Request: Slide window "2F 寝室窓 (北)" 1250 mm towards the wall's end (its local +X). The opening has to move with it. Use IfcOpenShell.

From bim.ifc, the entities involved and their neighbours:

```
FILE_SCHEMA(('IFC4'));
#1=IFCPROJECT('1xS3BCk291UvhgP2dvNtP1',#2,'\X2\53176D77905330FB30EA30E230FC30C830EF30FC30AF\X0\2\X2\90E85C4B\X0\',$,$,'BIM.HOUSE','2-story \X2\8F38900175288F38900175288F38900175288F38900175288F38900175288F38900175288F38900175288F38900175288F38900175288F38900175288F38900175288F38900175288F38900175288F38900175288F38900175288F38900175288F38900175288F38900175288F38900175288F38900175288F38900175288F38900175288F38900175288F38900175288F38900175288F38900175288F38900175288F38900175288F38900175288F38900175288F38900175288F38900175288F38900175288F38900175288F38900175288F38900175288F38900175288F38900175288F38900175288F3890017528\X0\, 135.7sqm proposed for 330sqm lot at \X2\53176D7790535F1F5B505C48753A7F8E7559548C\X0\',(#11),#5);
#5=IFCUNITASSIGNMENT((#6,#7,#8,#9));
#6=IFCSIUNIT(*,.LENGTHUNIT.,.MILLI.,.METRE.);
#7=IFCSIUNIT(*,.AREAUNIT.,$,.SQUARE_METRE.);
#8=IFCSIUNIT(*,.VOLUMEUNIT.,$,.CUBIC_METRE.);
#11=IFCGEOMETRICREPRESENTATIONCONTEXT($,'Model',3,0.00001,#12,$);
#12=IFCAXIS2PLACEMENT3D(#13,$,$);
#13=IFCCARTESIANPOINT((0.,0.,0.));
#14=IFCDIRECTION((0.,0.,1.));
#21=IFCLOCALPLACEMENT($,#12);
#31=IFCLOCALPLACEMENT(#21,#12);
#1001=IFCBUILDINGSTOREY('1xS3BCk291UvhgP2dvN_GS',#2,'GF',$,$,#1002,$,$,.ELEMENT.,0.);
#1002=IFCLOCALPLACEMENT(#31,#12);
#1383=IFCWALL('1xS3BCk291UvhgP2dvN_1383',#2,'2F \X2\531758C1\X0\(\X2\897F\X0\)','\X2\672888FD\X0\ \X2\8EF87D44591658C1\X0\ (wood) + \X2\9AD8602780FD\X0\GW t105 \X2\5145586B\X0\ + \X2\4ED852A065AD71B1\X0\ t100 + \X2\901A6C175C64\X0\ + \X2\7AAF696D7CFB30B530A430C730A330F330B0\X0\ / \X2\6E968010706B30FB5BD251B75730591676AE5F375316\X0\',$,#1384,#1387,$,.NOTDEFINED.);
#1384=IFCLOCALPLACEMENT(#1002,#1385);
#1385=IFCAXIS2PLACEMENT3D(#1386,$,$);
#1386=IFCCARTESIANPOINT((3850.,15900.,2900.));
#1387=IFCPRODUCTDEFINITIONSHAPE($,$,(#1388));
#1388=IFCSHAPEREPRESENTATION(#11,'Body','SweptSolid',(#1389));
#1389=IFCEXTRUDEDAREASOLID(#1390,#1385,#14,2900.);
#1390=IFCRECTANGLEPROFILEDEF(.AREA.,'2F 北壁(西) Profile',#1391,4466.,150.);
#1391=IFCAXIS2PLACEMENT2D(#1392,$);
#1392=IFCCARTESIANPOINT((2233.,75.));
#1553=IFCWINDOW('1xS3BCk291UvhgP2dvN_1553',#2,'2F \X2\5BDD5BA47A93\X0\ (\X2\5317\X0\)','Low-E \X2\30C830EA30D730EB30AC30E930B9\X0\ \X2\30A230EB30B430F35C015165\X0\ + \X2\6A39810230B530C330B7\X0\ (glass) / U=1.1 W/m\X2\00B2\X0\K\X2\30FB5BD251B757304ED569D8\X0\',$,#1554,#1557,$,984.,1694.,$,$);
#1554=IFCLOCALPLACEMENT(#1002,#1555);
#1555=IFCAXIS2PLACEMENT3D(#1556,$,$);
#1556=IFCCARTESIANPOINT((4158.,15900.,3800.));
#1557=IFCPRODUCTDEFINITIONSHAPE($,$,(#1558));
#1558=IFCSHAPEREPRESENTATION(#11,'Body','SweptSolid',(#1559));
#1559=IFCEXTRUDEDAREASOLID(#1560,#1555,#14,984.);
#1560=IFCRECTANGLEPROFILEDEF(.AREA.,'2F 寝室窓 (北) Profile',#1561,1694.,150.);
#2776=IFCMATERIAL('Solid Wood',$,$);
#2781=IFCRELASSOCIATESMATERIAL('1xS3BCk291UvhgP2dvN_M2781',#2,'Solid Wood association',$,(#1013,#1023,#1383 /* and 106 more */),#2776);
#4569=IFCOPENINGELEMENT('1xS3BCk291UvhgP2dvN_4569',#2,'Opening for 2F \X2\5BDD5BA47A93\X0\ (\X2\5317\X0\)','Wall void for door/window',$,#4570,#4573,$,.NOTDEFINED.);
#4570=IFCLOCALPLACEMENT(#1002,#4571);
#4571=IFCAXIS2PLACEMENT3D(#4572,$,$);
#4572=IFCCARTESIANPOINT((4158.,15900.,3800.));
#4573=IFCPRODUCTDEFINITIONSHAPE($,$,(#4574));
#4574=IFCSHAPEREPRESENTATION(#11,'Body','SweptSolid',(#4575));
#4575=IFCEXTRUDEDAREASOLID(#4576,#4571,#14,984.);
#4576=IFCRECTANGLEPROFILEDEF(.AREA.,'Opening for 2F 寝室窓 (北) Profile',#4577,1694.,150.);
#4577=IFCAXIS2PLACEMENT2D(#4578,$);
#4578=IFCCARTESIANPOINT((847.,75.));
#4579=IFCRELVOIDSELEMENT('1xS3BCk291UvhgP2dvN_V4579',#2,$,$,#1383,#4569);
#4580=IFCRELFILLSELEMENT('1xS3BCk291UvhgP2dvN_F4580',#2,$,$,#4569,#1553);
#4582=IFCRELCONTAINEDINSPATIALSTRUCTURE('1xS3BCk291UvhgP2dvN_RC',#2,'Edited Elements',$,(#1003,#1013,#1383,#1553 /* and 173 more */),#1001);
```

```python
import ifcopenshell
import ifcopenshell.api.geometry
import ifcopenshell.util.placement
import ifcopenshell.util.unit

model = ifcopenshell.open("bim.ifc")
unit_scale = ifcopenshell.util.unit.calculate_unit_scale(model)

window = model.by_id(1553)
opening = window.FillsVoids[0].RelatingOpeningElement
wall = opening.VoidsElements[0].RelatingBuildingElement

wall_matrix = ifcopenshell.util.placement.get_local_placement(wall.ObjectPlacement)
shift = wall_matrix[:3, 0] * 1.25 / unit_scale
before = ifcopenshell.util.placement.get_local_placement(window.ObjectPlacement)[:3, 3].copy()

# The window is not placed relative to its opening, so move both.
for product in (opening, window):
    matrix = ifcopenshell.util.placement.get_local_placement(product.ObjectPlacement)
    matrix[:3, 3] += shift
    ifcopenshell.api.geometry.edit_object_placement(model, product=product, matrix=matrix, is_si=False)

after = ifcopenshell.util.placement.get_local_placement(window.ObjectPlacement)[:3, 3]
print("window moved by", (after - before).round(3) + 0.0)

model.write("bim-out.ifc")
```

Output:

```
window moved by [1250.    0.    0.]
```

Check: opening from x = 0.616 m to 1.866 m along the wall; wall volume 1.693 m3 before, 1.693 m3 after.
